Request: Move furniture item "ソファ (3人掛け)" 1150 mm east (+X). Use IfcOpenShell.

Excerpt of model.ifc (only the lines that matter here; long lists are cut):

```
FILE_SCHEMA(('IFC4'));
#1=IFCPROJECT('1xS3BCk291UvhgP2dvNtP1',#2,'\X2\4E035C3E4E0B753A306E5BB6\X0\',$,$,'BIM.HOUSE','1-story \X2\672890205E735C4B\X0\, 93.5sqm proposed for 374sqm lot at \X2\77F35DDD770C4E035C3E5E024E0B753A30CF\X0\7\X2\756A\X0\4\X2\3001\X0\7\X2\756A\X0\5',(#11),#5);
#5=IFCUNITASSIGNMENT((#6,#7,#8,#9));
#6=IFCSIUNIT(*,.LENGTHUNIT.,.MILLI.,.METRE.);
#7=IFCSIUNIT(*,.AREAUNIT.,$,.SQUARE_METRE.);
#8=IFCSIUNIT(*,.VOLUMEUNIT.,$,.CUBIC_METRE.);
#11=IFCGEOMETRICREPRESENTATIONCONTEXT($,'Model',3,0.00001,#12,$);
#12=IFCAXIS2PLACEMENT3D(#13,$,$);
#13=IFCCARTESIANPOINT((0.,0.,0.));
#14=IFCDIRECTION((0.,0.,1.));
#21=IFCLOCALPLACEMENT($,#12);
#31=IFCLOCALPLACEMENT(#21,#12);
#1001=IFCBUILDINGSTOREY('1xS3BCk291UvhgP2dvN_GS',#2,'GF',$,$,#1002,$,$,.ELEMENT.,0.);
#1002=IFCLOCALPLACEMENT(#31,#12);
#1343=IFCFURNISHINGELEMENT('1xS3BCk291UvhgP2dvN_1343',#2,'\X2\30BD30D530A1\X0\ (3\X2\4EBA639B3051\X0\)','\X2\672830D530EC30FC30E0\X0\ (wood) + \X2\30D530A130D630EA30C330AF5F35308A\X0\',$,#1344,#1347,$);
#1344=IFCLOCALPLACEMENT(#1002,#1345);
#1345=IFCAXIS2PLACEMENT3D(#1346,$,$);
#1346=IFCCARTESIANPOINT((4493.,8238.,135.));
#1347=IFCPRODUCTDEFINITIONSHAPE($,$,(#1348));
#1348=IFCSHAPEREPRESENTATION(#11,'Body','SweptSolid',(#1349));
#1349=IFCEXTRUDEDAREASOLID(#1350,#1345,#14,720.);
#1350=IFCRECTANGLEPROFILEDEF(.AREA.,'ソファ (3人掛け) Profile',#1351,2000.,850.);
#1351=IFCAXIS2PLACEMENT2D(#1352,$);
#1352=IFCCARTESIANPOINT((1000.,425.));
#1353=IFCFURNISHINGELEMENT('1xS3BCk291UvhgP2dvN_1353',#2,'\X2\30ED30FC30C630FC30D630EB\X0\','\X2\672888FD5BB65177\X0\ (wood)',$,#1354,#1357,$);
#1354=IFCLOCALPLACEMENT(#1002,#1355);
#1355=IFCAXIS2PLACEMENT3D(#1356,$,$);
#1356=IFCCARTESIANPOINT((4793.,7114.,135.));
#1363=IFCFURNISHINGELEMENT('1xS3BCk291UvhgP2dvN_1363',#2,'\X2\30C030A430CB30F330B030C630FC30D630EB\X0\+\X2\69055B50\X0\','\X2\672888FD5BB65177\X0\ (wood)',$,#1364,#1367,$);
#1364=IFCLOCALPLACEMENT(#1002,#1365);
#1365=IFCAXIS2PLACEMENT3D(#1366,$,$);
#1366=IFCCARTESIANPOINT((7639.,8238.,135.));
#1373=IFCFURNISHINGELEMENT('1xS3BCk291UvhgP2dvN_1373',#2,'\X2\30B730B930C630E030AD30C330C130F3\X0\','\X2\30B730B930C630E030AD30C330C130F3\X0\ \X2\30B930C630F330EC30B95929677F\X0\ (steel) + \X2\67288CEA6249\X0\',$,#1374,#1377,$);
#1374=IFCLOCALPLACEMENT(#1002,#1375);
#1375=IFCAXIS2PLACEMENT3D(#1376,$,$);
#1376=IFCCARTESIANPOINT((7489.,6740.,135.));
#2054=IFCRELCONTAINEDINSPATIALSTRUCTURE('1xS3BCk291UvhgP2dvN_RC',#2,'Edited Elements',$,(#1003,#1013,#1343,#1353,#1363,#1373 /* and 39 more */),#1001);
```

```python
import ifcopenshell
import ifcopenshell.api.geometry
import ifcopenshell.util.placement
import ifcopenshell.util.unit

model = ifcopenshell.open("model.ifc")
unit_scale = ifcopenshell.util.unit.calculate_unit_scale(model)

item = model.by_id(1343)
matrix = ifcopenshell.util.placement.get_local_placement(item.ObjectPlacement)
matrix[0, 3] += 1.15 / unit_scale
ifcopenshell.api.geometry.edit_object_placement(model, product=item, matrix=matrix, is_si=False)

print(ifcopenshell.util.placement.get_local_placement(item.ObjectPlacement).round(3) + 0.0)

model.write("model_v2.ifc")
```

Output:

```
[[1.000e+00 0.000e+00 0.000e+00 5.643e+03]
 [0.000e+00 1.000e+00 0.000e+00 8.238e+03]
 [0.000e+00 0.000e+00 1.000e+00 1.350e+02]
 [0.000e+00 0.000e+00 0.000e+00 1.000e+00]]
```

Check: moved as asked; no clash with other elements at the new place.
